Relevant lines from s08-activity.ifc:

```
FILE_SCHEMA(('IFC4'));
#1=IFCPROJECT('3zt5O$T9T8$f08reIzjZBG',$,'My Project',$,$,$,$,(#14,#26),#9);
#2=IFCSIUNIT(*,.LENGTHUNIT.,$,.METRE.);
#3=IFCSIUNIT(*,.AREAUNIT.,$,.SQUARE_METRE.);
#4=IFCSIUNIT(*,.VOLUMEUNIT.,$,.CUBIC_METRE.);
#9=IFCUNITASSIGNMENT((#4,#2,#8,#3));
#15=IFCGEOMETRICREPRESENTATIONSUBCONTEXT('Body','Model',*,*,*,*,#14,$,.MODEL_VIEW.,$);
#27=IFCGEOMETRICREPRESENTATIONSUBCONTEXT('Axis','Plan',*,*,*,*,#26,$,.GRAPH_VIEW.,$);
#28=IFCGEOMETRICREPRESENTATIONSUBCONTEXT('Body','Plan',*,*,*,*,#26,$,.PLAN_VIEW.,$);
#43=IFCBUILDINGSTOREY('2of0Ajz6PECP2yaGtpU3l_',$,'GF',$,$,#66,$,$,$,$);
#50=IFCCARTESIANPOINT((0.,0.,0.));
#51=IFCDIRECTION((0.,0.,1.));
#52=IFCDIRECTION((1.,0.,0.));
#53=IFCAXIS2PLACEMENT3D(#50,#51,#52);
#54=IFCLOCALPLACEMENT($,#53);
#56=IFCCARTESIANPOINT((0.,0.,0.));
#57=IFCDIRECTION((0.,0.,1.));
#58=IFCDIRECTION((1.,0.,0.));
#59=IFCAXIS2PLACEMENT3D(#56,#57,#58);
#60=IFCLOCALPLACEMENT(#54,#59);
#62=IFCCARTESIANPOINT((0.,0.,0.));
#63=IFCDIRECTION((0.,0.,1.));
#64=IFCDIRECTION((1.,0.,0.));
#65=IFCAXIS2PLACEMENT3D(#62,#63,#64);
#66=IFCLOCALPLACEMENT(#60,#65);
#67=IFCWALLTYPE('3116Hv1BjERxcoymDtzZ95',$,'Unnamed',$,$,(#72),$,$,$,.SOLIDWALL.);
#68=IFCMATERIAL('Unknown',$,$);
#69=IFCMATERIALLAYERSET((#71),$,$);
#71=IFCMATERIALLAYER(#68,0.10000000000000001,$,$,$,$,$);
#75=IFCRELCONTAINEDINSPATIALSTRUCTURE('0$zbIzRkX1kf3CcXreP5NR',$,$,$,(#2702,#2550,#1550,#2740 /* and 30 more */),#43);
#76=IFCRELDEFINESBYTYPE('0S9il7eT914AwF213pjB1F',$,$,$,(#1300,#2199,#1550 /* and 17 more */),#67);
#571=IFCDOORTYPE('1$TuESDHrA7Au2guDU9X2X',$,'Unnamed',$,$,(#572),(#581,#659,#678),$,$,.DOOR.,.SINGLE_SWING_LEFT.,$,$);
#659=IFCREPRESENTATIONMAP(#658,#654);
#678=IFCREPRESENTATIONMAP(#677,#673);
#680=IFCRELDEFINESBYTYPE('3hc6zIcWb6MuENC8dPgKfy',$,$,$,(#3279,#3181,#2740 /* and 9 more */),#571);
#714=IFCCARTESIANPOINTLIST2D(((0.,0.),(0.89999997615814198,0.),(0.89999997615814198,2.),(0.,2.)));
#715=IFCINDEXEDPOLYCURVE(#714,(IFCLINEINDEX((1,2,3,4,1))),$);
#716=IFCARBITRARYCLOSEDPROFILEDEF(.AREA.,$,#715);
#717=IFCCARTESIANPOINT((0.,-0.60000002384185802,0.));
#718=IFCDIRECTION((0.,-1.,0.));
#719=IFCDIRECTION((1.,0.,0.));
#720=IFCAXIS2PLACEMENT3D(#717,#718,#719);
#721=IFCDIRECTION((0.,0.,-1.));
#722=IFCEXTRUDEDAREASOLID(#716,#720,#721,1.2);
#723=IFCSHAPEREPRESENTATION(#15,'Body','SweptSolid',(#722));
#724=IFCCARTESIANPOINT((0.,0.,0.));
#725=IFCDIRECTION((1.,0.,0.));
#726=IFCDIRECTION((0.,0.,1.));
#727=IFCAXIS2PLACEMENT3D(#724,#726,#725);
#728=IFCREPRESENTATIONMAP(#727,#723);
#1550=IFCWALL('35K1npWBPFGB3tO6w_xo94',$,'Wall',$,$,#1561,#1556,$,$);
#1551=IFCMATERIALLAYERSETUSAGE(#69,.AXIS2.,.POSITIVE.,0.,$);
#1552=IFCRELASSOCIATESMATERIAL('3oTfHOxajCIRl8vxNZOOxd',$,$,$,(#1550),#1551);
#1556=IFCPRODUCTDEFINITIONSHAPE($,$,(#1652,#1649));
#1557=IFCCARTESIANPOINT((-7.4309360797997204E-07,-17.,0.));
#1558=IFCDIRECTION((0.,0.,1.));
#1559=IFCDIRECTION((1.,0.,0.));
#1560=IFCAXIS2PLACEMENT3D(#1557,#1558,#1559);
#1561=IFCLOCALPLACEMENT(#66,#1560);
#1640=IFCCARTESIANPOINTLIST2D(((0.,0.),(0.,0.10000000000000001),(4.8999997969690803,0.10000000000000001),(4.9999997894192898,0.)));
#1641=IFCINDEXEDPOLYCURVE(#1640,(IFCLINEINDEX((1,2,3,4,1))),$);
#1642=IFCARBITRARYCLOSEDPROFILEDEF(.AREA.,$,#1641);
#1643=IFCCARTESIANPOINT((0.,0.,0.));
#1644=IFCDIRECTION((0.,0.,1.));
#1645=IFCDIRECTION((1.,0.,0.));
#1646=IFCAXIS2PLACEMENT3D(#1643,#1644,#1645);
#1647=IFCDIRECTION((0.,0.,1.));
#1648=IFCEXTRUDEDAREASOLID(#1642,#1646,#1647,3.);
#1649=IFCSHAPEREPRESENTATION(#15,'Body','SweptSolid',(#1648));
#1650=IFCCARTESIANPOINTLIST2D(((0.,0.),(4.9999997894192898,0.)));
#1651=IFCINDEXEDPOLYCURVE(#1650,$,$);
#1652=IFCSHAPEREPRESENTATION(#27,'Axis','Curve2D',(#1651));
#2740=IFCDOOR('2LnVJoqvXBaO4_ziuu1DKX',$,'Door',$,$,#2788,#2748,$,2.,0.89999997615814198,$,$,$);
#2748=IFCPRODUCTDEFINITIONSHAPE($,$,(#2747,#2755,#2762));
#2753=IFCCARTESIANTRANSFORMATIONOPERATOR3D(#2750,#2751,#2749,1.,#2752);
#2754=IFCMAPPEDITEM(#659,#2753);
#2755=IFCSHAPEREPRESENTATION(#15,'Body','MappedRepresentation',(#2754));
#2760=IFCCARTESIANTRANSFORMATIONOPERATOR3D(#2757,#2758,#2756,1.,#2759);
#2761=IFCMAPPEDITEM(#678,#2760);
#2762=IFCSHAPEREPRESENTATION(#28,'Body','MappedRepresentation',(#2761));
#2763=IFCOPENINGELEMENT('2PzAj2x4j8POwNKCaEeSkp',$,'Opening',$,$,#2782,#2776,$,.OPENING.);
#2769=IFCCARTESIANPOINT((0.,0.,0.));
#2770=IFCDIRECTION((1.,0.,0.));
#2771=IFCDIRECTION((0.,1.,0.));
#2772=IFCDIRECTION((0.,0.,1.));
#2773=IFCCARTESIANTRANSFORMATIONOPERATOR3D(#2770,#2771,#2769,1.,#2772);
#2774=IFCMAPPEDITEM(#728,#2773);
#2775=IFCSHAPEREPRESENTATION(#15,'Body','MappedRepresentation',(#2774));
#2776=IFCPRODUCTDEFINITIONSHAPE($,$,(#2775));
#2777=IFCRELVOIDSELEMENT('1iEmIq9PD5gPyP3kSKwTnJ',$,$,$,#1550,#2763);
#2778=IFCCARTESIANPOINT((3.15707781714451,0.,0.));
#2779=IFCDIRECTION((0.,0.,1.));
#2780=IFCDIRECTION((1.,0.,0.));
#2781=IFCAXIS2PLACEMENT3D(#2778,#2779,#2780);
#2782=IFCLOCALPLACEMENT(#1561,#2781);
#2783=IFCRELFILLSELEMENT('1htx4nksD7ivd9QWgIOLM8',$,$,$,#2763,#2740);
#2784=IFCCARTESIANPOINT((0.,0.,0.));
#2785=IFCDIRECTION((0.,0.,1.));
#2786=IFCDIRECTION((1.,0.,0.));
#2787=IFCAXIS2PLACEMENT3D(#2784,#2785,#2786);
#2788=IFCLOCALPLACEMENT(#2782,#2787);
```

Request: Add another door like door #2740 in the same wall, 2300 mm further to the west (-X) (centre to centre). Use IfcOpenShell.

```python
import ifcopenshell
import ifcopenshell.api.feature
import ifcopenshell.api.geometry
import ifcopenshell.api.root
import ifcopenshell.geom
import ifcopenshell.util.element
import ifcopenshell.util.placement
import ifcopenshell.util.shape

model = ifcopenshell.open("s08-activity.ifc")
settings = ifcopenshell.geom.settings()


def volume(element):
    """Net volume in cubic metres, openings subtracted."""
    shape = ifcopenshell.geom.create_shape(settings, element)
    return ifcopenshell.util.shape.get_volume(shape.geometry)


door = model.by_guid("2LnVJoqvXBaO4_ziuu1DKX")
opening = door.FillsVoids[0].RelatingOpeningElement
wall = opening.VoidsElements[0].RelatingBuildingElement
before = volume(wall)
shift = ifcopenshell.util.placement.get_local_placement(wall.ObjectPlacement)[:3, 0] * -2.3

# copy_class copies the void relationship, type, container and properties, but no geometry.
new_opening = ifcopenshell.api.root.copy_class(model, product=opening)
new_opening.Representation = ifcopenshell.util.element.copy_deep(
    model, opening.Representation, exclude=["IfcGeometricRepresentationContext", "IfcRepresentationMap"]
)
new_door = ifcopenshell.api.root.copy_class(model, product=door)
new_door.Representation = ifcopenshell.util.element.copy_deep(
    model, door.Representation, exclude=["IfcGeometricRepresentationContext", "IfcRepresentationMap"]
)
ifcopenshell.api.feature.add_filling(model, opening=new_opening, element=new_door)

for old, new in ((opening, new_opening), (door, new_door)):
    matrix = ifcopenshell.util.placement.get_local_placement(old.ObjectPlacement)
    matrix[:3, 3] += shift
    ifcopenshell.api.geometry.edit_object_placement(model, product=new, matrix=matrix, is_si=False)

after = volume(wall)

print(f"wall volume {before:.3f} -> {after:.3f} m3")

model.write("s08-activity-out.ifc")
```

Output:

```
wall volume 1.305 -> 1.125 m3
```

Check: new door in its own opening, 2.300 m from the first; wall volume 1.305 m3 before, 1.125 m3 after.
